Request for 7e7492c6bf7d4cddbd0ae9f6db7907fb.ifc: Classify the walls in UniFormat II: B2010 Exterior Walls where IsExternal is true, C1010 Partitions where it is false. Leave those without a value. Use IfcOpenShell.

First a look at what the model holds.

```python
import ifcopenshell
import ifcopenshell.util.element

model = ifcopenshell.open("7e7492c6bf7d4cddbd0ae9f6db7907fb.ifc")
print(model.schema)
print("classifications:", [c.Name for c in model.by_type("IfcClassification")])
values = [ifcopenshell.util.element.get_pset(e, "Pset_WallCommon", "IsExternal") for e in model.by_type("IfcWall")]
for value in (True, False, None):
    print("IsExternal", value, values.count(value))
```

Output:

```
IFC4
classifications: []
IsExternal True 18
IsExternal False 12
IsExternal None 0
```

```python
import ifcopenshell
import ifcopenshell.api.classification
import ifcopenshell.util.element

model = ifcopenshell.open("7e7492c6bf7d4cddbd0ae9f6db7907fb.ifc")

system = ifcopenshell.api.classification.add_classification(model, classification="UniFormat II")

walls = model.by_type("IfcWall")
external = {e: ifcopenshell.util.element.get_pset(e, "Pset_WallCommon", "IsExternal") for e in walls}
for flag, code, name in ((True, "B2010", "Exterior Walls"), (False, "C1010", "Partitions")):
    products = [e for e in walls if external[e] is flag]
    ifcopenshell.api.classification.add_reference(
        model, products=products, classification=system, identification=code, name=name
    )
    print(code, len(products))

model.write("7e7492c6bf7d4cddbd0ae9f6db7907fb-out.ifc")
```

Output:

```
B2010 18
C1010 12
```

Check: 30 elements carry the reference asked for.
